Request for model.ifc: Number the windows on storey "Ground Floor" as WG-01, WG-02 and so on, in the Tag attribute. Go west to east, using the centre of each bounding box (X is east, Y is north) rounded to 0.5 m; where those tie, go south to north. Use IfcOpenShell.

First a look at what the model holds.

```python
import ifcopenshell
import ifcopenshell.util.element
import ifcopenshell.util.placement

model = ifcopenshell.open("model.ifc")
print(model.schema)
storey = next(s for s in model.by_type("IfcBuildingStorey") if s.Name == "Ground Floor")
windows = [e for e in ifcopenshell.util.element.get_decomposition(storey) if e.is_a("IfcWindow")]
for e in sorted(windows, key=lambda e: e.id()):
    origin = ifcopenshell.util.placement.get_local_placement(e.ObjectPlacement)[:3, 3]
    print(e.id(), e.Tag, e.Name, origin.round(2) + 0.0, sep=" | ")
```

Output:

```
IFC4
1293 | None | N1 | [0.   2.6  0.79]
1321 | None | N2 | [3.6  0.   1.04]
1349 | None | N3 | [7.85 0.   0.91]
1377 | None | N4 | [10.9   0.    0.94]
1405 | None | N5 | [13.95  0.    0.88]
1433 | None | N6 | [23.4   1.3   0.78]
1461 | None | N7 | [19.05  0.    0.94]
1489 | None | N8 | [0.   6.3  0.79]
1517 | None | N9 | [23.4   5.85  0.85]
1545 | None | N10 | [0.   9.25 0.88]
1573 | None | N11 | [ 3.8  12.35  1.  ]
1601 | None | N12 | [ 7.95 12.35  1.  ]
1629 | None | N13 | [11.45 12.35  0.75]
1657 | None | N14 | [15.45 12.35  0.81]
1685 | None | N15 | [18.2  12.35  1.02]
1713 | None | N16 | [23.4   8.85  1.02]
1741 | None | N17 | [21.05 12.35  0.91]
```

```python
import ifcopenshell
import ifcopenshell.geom
import ifcopenshell.util.element
import ifcopenshell.util.shape

model = ifcopenshell.open("model.ifc")
settings = ifcopenshell.geom.settings()
settings.set("use-world-coords", True)


def centre(element):
    shape = ifcopenshell.geom.create_shape(settings, element)
    return ifcopenshell.util.shape.get_bbox_centroid(shape.geometry)


storey = next(s for s in model.by_type("IfcBuildingStorey") if s.Name == "Ground Floor")
windows = [e for e in ifcopenshell.util.element.get_decomposition(storey) if e.is_a("IfcWindow")]

# Insertion points can sit at a corner or the storey origin, so sort by the geometry (in metres).
centres = {e: centre(e) for e in windows}
windows.sort(key=lambda e: (round(centres[e][0] / 0.5), centres[e][1]))

for i, e in enumerate(windows, start=1):
    number = f"WG-{i:02d}"
    e.Tag = number
    print(e.id(), number)

model.write("model_updated.ifc")
```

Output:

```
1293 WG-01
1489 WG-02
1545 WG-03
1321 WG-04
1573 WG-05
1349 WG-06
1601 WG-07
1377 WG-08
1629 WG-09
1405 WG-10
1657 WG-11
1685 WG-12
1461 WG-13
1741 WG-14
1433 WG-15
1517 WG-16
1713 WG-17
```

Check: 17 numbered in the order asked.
